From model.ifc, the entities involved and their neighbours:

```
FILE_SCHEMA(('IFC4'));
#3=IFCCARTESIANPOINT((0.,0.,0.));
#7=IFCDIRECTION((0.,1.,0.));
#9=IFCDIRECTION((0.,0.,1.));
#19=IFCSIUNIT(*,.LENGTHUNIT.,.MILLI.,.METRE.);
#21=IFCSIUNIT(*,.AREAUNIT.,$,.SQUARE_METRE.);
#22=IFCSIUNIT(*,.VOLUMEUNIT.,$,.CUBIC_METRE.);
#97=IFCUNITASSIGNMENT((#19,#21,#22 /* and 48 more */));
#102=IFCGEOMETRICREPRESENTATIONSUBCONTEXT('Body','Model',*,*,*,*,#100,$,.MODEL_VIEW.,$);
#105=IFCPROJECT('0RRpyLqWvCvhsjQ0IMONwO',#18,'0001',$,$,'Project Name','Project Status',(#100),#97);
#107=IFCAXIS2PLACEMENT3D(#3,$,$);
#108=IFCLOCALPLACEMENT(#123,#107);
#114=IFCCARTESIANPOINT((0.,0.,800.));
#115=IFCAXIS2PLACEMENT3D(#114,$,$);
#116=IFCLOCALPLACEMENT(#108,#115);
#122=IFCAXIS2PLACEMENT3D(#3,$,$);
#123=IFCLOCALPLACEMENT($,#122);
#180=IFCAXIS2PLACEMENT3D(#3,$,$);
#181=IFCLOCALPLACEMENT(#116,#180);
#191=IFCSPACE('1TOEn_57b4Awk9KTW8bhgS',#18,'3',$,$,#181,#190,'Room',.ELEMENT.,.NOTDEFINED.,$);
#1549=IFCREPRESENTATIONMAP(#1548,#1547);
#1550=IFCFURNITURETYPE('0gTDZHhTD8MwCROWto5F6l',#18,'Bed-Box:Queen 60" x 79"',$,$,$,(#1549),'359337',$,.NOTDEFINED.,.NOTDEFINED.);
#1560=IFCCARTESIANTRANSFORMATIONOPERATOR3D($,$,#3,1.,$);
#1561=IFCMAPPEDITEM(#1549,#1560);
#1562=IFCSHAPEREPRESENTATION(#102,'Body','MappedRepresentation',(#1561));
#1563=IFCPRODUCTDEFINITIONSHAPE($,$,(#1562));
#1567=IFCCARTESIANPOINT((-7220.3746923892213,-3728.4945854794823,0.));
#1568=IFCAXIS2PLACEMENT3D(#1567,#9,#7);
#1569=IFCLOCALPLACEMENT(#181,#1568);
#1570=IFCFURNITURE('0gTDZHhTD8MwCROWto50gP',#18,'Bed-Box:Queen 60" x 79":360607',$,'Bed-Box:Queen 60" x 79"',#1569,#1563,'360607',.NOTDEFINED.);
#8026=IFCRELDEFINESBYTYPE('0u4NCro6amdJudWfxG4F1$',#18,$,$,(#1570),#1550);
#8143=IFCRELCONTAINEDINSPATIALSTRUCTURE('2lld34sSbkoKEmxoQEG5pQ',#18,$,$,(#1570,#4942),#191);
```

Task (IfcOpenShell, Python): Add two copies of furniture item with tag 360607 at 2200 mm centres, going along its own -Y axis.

```python
import ifcopenshell
import ifcopenshell.api.geometry
import ifcopenshell.api.root
import ifcopenshell.util.element
import ifcopenshell.util.placement
import ifcopenshell.util.unit

model = ifcopenshell.open("model.ifc")
unit_scale = ifcopenshell.util.unit.calculate_unit_scale(model)


def reuse_history(source, copy):
    """copy_class also copies each property set's owner history, people and application; keep the originals."""
    for rel in copy.IsDefinedBy:
        if rel.is_a("IfcRelDefinesByProperties") and (history := rel.RelatingPropertyDefinition.OwnerHistory):
            rel.RelatingPropertyDefinition.OwnerHistory = source.OwnerHistory
            ifcopenshell.util.element.remove_deep2(model, history)


source = model.by_id(1570)
base = ifcopenshell.util.placement.get_local_placement(source.ObjectPlacement)
step = -base[:3, 1] * 2.2 / unit_scale

for i in range(1, 3):
    copy = ifcopenshell.api.root.copy_class(model, product=source)
    copy.Representation = ifcopenshell.util.element.copy_deep(
        model, source.Representation, exclude=["IfcGeometricRepresentationContext", "IfcRepresentationMap"]
    )
    copy.Name = 'Bed-Box:Queen 60" x 79"'
    copy.Tag = None
    reuse_history(source, copy)
    matrix = base.copy()
    matrix[:3, 3] += i * step
    print("added at", matrix[:3, 3].round(3) + 0.0)
    ifcopenshell.api.geometry.edit_object_placement(model, product=copy, matrix=matrix, is_si=False)

model.write("model_v2.ifc")
```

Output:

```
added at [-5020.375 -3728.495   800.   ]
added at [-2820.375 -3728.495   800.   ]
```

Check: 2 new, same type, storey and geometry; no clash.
